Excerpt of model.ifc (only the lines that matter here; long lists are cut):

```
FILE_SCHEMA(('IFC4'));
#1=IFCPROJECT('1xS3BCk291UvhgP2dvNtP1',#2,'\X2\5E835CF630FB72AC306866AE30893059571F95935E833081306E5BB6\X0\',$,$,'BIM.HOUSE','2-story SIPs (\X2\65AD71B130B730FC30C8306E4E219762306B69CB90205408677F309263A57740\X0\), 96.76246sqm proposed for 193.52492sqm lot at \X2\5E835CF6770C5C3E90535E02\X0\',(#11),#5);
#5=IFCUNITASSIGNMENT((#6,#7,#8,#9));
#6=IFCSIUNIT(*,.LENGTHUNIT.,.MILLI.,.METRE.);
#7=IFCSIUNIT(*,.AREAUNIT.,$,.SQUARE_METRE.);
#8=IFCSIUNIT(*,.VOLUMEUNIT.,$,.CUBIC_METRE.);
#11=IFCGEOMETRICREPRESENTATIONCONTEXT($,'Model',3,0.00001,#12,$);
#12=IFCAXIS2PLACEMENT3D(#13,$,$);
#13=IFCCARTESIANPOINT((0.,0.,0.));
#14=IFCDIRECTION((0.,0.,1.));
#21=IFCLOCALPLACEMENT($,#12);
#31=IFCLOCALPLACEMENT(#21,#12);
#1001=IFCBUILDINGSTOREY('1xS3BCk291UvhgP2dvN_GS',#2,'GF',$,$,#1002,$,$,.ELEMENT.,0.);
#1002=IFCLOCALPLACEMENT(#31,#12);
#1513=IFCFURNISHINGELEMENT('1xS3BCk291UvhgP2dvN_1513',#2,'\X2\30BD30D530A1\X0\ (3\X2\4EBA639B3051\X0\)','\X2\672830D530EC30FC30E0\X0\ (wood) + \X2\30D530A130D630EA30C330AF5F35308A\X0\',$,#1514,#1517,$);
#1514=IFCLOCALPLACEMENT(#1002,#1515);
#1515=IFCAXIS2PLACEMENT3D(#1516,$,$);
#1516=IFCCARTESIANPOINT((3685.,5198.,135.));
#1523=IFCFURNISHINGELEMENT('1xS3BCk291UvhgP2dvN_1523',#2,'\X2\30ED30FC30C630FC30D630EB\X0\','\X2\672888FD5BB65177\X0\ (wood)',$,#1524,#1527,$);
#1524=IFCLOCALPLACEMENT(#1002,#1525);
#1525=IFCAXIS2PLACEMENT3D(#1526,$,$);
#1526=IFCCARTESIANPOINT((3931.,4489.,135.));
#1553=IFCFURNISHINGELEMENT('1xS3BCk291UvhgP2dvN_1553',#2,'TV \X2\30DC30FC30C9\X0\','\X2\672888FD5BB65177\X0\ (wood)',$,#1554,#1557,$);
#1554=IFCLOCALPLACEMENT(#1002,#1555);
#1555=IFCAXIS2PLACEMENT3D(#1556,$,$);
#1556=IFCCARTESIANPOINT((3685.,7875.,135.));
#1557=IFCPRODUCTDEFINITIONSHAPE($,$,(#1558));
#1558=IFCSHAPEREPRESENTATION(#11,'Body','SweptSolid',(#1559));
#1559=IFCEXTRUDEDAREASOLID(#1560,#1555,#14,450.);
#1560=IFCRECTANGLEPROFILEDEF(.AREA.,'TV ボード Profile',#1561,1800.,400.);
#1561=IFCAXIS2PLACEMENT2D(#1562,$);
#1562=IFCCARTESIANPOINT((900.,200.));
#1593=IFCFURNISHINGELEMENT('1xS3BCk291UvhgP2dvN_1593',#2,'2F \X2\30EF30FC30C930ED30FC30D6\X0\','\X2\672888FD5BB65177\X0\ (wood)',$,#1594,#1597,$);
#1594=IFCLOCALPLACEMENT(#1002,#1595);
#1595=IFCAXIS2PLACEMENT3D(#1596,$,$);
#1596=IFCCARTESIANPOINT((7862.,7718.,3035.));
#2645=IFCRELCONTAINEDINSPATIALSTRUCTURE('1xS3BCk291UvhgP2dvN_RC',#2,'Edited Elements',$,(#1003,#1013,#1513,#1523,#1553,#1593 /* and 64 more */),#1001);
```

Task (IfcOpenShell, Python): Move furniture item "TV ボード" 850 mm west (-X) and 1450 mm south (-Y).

```python
import ifcopenshell
import ifcopenshell.api.geometry
import ifcopenshell.util.placement

model = ifcopenshell.open("model.ifc")

item = model.by_id(1553)
matrix = ifcopenshell.util.placement.get_local_placement(item.ObjectPlacement)
matrix[0, 3] -= 850.0
matrix[1, 3] -= 1450.0
ifcopenshell.api.geometry.edit_object_placement(model, product=item, matrix=matrix, is_si=False)

print(ifcopenshell.util.placement.get_local_placement(item.ObjectPlacement).round(3) + 0.0)

model.write("model_rev.ifc")
```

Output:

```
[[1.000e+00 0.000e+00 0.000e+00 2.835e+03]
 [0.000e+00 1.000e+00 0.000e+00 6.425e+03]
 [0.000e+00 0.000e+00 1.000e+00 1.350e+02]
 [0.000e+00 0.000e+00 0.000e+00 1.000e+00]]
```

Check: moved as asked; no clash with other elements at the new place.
